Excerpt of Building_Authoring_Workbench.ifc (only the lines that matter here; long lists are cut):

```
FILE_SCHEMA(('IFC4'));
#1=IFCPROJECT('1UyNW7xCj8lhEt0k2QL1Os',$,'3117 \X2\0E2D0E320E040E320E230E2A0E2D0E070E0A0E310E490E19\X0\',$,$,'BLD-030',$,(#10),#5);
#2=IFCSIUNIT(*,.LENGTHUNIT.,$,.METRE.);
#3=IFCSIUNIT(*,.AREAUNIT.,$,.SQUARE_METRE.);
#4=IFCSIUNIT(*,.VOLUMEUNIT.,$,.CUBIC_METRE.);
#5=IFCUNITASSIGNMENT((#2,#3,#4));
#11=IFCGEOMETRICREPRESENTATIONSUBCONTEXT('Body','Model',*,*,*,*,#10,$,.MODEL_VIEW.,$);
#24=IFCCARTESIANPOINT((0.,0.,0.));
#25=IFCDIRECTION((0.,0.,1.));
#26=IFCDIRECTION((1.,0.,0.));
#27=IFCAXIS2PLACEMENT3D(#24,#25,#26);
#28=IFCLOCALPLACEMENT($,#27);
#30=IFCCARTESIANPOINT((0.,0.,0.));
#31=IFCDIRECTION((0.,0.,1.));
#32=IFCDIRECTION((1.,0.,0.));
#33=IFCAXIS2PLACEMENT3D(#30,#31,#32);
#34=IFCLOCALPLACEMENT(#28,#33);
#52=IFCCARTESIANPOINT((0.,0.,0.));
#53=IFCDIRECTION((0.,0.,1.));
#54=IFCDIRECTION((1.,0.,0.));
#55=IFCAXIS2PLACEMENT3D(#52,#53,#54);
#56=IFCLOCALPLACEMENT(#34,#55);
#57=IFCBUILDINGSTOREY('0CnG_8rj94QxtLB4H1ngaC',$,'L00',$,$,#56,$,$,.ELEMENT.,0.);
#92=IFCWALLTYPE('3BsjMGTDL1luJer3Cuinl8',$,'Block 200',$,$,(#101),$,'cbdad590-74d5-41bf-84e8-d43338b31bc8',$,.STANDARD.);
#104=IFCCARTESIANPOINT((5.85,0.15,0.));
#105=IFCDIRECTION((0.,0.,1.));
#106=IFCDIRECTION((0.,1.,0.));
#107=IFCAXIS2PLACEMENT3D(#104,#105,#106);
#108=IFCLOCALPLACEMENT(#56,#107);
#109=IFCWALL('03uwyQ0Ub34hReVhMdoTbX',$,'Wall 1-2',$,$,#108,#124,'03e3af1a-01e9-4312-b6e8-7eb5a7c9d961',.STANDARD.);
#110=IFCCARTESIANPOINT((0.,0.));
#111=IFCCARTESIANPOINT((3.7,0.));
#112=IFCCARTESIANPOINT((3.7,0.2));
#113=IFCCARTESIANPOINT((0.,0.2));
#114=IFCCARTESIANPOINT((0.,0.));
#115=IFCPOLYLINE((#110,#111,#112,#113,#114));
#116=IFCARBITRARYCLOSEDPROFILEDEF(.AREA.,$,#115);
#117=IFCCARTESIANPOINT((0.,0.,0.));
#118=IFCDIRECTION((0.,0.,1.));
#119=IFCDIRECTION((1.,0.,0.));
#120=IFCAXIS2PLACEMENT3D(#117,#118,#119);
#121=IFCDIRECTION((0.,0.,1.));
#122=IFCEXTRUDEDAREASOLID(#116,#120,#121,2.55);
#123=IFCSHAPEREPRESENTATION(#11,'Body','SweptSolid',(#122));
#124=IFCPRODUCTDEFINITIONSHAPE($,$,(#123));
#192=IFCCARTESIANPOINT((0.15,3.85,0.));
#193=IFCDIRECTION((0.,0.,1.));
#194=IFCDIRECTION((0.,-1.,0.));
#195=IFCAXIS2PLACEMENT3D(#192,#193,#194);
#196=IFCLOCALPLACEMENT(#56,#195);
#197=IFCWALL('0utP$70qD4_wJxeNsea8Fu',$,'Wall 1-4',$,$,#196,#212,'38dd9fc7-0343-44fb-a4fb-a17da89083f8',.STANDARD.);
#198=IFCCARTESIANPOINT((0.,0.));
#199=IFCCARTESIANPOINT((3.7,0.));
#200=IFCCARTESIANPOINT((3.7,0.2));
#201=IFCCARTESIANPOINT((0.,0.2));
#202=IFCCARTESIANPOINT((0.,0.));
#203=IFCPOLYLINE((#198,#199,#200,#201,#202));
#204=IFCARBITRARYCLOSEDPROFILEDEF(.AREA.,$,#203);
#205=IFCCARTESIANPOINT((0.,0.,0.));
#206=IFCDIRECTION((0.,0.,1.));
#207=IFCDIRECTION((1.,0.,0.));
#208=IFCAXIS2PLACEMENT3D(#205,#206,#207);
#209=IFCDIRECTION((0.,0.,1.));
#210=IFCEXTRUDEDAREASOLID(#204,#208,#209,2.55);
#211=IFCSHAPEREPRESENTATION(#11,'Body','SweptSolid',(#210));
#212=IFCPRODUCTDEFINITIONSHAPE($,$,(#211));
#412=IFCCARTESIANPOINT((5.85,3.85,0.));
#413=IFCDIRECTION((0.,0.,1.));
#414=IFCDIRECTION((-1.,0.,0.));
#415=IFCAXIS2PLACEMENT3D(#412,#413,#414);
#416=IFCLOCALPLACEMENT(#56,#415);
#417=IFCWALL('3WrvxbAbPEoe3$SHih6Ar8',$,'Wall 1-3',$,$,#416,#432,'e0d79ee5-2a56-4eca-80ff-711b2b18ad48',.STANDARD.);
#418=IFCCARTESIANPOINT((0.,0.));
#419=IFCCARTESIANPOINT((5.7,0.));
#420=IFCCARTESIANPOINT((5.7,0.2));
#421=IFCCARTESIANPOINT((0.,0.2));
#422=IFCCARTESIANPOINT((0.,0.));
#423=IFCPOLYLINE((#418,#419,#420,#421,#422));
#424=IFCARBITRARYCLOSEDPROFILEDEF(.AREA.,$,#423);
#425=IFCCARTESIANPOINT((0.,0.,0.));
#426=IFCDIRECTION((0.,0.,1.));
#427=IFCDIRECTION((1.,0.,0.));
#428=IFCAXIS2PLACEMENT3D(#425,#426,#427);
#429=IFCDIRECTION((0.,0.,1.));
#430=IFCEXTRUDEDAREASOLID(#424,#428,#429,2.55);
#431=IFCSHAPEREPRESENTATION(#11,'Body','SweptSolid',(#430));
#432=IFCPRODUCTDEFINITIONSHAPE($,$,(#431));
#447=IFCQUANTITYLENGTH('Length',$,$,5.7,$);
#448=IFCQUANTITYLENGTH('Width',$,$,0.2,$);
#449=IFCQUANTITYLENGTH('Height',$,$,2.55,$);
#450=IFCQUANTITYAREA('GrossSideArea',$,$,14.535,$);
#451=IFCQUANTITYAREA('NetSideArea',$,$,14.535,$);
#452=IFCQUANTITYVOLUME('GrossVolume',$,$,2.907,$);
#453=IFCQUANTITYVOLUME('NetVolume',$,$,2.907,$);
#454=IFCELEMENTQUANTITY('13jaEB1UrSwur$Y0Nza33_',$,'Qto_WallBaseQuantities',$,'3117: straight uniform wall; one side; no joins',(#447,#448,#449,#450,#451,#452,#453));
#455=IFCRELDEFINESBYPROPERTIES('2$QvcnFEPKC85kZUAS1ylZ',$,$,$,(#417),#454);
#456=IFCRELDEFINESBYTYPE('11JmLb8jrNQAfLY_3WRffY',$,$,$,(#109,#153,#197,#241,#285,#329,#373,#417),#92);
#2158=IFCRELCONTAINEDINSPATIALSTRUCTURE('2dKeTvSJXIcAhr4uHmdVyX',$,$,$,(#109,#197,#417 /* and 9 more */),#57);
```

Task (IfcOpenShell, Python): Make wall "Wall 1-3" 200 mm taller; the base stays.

```python
import ifcopenshell
import ifcopenshell.api.pset
import ifcopenshell.geom
import ifcopenshell.util.element
import ifcopenshell.util.representation
import ifcopenshell.util.shape
import ifcopenshell.util.unit

model = ifcopenshell.open("Building_Authoring_Workbench.ifc")
unit_scale = ifcopenshell.util.unit.calculate_unit_scale(model)
area_scale = ifcopenshell.util.unit.calculate_unit_scale(model, "AREAUNIT")
volume_scale = ifcopenshell.util.unit.calculate_unit_scale(model, "VOLUMEUNIT")
settings = ifcopenshell.geom.settings()


def volume(element):
    """Net volume in cubic metres, openings subtracted."""
    shape = ifcopenshell.geom.create_shape(settings, element)
    return ifcopenshell.util.shape.get_volume(shape.geometry)


wall = model.by_guid("3WrvxbAbPEoe3$SHih6Ar8")
before = volume(wall)

body = ifcopenshell.util.representation.get_representation(wall, "Model", "Body")
solid = body.Items[0]
old_height = solid.Depth
solid.Depth += 0.2
after = volume(wall)
thickness = 0.2  # wall thickness in metres

# Update the stored height, areas and volumes.
qto = model.by_id(ifcopenshell.util.element.get_pset(wall, "Qto_WallBaseQuantities", should_inherit=False)["id"])
ifcopenshell.api.pset.edit_qto(model, qto=qto, properties={
    "Height": solid.Depth,
    "GrossSideArea": ifcopenshell.util.element.get_pset(wall, "Qto_WallBaseQuantities", "GrossSideArea") * solid.Depth / old_height,
    "NetSideArea": after / thickness / area_scale,
    "GrossVolume": ifcopenshell.util.element.get_pset(wall, "Qto_WallBaseQuantities", "GrossVolume") * solid.Depth / old_height,
    "NetVolume": after / volume_scale,
})

print(f"height {old_height:g} -> {solid.Depth:g}, volume {before:.3f} -> {after:.3f} m3")

model.write("Building_Authoring_Workbench_v2.ifc")
```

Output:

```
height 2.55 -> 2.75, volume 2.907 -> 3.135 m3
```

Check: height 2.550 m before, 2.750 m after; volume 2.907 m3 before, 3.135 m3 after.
